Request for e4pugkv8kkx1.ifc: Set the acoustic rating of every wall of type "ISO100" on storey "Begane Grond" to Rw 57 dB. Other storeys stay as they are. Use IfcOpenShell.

First a look at what the model holds.

```python
import ifcopenshell
import ifcopenshell.util.element

model = ifcopenshell.open("e4pugkv8kkx1.ifc")
print(model.schema)
storey = next(s for s in model.by_type("IfcBuildingStorey") if s.Name == "Begane Grond")
walls = [e for e in ifcopenshell.util.element.get_decomposition(storey) if e.is_a("IfcWall")]
seen = {}
for e in walls:
    element_type = ifcopenshell.util.element.get_type(e)
    key = (element_type.Name if element_type != e and element_type else None, ifcopenshell.util.element.get_pset(e, "Pset_WallCommon", "AcousticRating"))
    seen[key] = seen.get(key, 0) + 1
for (name, value), count in sorted(seen.items(), key=str):
    print(count, "x", name, "|", value)
```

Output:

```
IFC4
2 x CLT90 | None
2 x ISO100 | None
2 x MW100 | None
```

```python
import ifcopenshell
import ifcopenshell.api.pset
import ifcopenshell.util.element

model = ifcopenshell.open("e4pugkv8kkx1.ifc")

storey = next(s for s in model.by_type("IfcBuildingStorey") if s.Name == "Begane Grond")
walls = [e for e in ifcopenshell.util.element.get_decomposition(storey) if e.is_a("IfcWall")]

count = 0
for e in walls:
    element_type = ifcopenshell.util.element.get_type(e)
    if element_type in (None, e) or element_type.Name != "ISO100":
        continue
    # add_pset returns the element's existing set when there is one.
    pset = ifcopenshell.api.pset.add_pset(model, product=e, name="Pset_WallCommon")
    ifcopenshell.api.pset.edit_pset(model, pset=pset, properties={"AcousticRating": "Rw 57 dB"})
    count += 1

print(count, "walls updated")

model.write("e4pugkv8kkx1_v2.ifc")
```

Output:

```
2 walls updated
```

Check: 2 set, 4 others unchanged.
